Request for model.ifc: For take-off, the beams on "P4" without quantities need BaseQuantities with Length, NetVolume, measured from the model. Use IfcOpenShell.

First a look at what the model holds.

```python
import ifcopenshell
import ifcopenshell.util.element
import ifcopenshell.util.unit

model = ifcopenshell.open("model.ifc")
print(model.schema)
for unit_type in ("LENGTHUNIT", "AREAUNIT", "VOLUMEUNIT"):
    print(unit_type, ifcopenshell.util.unit.calculate_unit_scale(model, unit_type))
storey = next(s for s in model.by_type("IfcBuildingStorey") if s.Name == "P4")
beams = [e for e in ifcopenshell.util.element.get_decomposition(storey) if e.is_a("IfcBeam")]
for e in sorted(beams, key=lambda e: e.id()):
    print(e.id(), e.is_a(), e.Name, list(ifcopenshell.util.element.get_psets(e, qtos_only=True)), sep=" | ")
```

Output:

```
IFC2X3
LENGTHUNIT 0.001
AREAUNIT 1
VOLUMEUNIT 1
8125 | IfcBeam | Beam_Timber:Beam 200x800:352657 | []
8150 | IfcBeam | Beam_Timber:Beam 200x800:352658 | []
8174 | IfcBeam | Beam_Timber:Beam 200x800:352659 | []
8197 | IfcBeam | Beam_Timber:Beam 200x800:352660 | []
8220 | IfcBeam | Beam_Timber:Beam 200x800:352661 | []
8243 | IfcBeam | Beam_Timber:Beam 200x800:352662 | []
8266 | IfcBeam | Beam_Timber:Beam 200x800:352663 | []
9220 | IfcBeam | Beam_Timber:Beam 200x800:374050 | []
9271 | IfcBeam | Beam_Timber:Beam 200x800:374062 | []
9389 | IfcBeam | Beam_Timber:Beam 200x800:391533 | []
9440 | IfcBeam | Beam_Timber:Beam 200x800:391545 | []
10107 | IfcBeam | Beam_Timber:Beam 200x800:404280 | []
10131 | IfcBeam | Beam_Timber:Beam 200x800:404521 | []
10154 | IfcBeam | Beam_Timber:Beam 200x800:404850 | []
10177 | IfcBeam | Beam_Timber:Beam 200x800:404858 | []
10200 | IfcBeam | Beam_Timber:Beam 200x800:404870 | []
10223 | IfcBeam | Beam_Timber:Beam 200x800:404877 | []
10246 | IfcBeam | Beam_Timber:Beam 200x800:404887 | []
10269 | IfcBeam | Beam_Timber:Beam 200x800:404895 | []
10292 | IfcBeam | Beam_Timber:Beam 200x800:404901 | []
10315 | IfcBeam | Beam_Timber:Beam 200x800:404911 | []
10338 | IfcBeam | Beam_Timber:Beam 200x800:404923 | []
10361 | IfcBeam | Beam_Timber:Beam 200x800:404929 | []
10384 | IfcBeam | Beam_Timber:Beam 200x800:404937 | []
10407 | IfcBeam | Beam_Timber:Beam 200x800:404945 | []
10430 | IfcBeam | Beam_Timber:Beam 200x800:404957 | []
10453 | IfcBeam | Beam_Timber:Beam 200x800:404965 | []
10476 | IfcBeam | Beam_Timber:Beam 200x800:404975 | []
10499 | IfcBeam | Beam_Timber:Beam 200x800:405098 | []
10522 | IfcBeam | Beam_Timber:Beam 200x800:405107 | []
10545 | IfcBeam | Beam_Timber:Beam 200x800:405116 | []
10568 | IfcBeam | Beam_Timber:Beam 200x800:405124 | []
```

```python
import ifcopenshell
import ifcopenshell.api.pset
import ifcopenshell.geom
import ifcopenshell.util.element
import ifcopenshell.util.shape
import ifcopenshell.util.unit

model = ifcopenshell.open("model.ifc")
unit_scale = ifcopenshell.util.unit.calculate_unit_scale(model)
volume_scale = ifcopenshell.util.unit.calculate_unit_scale(model, "VOLUMEUNIT")
settings = ifcopenshell.geom.settings()

storey = next(s for s in model.by_type("IfcBuildingStorey") if s.Name == "P4")
beams = [e for e in ifcopenshell.util.element.get_decomposition(storey) if e.is_a("IfcBeam")]

for e in sorted(beams, key=lambda e: e.id()):
    if ifcopenshell.util.element.get_psets(e, qtos_only=True, should_inherit=False):
        continue
    # Geometry comes back in metres, in the element's own axes.
    shape = ifcopenshell.geom.create_shape(settings, e)
    values = {
        "Length": ifcopenshell.util.shape.get_max_xyz(shape.geometry) / unit_scale,
        "NetVolume": ifcopenshell.util.shape.get_volume(shape.geometry) / volume_scale,
    }
    qto = ifcopenshell.api.pset.add_qto(model, product=e, name="BaseQuantities")
    ifcopenshell.api.pset.edit_qto(model, qto=qto, properties=values)
    print(e.id(), {k: round(v, 3) for k, v in values.items()})

model.write("model_edited.ifc")
```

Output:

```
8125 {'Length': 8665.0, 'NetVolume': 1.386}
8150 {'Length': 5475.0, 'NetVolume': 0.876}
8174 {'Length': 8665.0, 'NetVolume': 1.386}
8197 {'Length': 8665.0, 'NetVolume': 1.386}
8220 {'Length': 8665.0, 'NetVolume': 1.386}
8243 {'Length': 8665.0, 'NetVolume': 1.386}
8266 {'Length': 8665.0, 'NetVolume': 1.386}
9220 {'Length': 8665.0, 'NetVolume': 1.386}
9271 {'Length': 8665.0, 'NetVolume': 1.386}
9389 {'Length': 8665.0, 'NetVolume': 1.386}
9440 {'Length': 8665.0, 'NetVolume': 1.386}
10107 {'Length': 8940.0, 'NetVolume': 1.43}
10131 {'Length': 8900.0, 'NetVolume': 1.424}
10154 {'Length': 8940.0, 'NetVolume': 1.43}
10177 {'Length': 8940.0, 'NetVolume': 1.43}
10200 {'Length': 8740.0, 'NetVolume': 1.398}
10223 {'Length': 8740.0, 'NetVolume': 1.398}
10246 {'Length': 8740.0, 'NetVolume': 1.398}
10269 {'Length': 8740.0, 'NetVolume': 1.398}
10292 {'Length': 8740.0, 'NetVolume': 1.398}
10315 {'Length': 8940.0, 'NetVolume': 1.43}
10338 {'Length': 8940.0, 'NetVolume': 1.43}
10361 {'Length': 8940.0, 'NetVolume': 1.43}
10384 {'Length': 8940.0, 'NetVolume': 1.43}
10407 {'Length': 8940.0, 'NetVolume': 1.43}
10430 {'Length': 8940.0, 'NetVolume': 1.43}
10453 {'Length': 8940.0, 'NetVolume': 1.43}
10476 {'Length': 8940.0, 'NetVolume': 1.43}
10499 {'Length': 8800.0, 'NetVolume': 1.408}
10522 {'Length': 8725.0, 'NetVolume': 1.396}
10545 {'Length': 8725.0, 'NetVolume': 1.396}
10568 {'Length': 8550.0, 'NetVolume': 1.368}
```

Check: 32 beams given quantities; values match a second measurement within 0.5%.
